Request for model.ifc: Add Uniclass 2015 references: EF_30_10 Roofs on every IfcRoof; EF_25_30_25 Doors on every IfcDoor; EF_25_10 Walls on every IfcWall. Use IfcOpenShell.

First a look at what the model holds.

```python
import ifcopenshell

model = ifcopenshell.open("model.ifc")
print(model.schema)
print("classifications:", [c.Name for c in model.by_type("IfcClassification")])
for ifc_class in ("IfcDoor", "IfcRoof", "IfcStair", "IfcWall", "IfcWindow"):
    print(ifc_class, len(model.by_type(ifc_class)))
```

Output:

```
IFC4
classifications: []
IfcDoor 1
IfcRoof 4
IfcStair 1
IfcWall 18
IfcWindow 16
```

```python
import ifcopenshell
import ifcopenshell.api.classification

model = ifcopenshell.open("model.ifc")

system = ifcopenshell.api.classification.add_classification(model, classification="Uniclass 2015")

codes = {
    "IfcRoof": ("EF_30_10", "Roofs"),
    "IfcDoor": ("EF_25_30_25", "Doors"),
    "IfcWall": ("EF_25_10", "Walls"),
}
for ifc_class, (code, name) in codes.items():
    products = model.by_type(ifc_class)
    ifcopenshell.api.classification.add_reference(
        model, products=products, classification=system, identification=code, name=name
    )
    print(code, len(products))

model.write("model-out.ifc")
```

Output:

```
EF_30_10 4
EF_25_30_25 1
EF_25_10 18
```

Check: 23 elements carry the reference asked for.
